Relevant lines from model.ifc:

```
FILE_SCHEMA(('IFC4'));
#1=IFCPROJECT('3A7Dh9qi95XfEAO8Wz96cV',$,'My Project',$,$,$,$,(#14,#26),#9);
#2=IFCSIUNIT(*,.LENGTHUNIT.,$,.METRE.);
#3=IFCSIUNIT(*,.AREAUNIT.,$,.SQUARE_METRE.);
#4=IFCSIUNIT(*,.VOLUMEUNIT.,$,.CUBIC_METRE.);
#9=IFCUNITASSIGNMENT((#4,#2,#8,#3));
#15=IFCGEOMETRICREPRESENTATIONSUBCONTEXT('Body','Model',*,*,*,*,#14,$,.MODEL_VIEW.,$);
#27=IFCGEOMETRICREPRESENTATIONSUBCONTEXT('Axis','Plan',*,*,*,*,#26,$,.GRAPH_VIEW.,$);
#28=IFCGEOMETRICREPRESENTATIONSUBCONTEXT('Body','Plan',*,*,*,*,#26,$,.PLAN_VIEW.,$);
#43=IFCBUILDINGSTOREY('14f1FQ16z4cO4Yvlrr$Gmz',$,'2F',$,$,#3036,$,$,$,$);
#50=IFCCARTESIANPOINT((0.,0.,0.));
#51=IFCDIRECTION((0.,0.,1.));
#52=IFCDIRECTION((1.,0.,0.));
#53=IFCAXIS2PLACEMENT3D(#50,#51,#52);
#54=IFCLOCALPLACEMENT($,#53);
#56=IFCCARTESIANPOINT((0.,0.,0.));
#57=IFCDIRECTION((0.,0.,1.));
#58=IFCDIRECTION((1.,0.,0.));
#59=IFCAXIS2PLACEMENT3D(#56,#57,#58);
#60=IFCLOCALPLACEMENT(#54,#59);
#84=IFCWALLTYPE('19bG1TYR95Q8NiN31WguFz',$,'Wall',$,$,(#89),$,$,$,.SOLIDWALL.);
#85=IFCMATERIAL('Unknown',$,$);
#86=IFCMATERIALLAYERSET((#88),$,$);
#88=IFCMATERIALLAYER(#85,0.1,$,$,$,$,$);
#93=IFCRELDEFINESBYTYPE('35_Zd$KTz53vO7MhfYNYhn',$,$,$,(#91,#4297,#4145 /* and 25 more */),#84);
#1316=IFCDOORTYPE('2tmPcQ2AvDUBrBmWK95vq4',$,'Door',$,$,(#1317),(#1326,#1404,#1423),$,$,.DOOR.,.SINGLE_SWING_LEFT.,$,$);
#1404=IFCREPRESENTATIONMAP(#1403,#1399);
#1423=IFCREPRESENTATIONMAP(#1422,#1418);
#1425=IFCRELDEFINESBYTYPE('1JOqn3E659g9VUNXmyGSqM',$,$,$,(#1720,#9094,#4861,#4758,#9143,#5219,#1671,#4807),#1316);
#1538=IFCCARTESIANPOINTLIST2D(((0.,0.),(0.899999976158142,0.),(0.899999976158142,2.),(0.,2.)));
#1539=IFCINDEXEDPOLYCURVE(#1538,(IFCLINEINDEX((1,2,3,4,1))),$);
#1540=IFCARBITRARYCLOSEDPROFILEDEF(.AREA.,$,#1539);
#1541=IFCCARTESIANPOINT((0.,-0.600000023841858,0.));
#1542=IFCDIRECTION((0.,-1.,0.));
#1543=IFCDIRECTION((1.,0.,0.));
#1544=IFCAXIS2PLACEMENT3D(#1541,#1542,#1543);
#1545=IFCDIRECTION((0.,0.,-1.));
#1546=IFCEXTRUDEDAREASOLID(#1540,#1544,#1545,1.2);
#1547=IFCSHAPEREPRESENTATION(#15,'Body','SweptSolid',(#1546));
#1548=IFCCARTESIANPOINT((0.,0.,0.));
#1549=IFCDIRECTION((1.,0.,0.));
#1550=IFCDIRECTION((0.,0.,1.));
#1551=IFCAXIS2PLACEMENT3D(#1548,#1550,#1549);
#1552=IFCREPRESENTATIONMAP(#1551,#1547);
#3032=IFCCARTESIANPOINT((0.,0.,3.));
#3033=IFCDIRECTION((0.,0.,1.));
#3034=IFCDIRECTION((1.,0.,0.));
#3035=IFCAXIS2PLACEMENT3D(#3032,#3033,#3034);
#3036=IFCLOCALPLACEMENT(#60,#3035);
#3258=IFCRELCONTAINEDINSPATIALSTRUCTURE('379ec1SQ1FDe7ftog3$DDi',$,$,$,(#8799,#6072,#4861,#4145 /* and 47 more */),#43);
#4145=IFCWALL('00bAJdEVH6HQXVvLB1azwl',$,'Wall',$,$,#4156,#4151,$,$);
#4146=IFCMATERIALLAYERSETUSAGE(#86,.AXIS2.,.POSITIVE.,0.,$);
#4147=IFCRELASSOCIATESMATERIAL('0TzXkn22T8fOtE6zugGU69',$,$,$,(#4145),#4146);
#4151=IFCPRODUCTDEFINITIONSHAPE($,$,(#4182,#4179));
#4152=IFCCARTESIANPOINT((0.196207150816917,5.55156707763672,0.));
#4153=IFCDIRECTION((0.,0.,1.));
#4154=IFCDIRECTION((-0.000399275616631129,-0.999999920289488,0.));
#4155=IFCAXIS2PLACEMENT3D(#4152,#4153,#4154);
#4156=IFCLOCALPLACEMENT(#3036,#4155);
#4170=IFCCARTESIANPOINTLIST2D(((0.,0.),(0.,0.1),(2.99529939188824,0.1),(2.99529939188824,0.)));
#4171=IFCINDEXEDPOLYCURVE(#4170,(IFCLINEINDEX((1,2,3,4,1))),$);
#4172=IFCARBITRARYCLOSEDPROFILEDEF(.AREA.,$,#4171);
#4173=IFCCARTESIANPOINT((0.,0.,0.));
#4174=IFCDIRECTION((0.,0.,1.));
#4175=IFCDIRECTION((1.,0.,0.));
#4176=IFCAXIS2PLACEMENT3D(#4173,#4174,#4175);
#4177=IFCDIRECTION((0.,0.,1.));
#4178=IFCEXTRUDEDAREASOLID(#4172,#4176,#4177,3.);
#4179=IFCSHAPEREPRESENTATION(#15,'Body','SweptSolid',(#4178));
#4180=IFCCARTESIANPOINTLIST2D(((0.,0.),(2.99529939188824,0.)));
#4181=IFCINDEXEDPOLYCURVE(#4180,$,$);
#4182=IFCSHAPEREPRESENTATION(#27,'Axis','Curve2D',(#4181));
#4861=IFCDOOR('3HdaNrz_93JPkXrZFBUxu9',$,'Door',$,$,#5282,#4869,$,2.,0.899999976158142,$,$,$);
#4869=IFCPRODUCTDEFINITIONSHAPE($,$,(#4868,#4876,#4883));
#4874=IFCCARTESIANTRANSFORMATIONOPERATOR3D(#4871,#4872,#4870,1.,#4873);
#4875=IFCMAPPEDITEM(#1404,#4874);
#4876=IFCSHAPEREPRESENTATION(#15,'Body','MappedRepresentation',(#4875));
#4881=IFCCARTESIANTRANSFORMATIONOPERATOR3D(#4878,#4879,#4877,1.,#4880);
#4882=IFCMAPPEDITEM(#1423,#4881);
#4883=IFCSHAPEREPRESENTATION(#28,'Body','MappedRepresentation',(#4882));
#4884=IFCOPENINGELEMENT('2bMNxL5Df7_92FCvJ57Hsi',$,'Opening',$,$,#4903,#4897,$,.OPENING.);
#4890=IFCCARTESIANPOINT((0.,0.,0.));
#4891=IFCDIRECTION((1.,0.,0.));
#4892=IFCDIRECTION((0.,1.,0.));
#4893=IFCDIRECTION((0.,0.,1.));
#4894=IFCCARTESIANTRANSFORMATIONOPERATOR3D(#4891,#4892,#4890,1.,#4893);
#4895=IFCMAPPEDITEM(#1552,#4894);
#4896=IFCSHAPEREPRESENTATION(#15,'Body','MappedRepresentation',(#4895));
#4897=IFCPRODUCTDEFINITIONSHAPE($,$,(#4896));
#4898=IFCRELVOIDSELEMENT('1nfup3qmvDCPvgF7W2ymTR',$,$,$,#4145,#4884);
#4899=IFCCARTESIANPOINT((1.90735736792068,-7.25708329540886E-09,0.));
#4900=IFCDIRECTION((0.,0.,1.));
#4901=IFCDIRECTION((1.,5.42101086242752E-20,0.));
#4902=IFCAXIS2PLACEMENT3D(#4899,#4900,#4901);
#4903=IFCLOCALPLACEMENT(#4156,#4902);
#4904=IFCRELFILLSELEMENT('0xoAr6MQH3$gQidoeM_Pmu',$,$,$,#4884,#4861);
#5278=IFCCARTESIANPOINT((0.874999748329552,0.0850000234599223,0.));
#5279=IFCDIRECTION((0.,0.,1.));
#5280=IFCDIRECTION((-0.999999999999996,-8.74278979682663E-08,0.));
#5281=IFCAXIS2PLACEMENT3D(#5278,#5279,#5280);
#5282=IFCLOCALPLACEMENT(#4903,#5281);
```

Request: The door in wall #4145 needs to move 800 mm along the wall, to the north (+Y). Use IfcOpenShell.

```python
import ifcopenshell
import ifcopenshell.api.geometry
import ifcopenshell.util.placement
import ifcopenshell.util.unit

model = ifcopenshell.open("model.ifc")
unit_scale = ifcopenshell.util.unit.calculate_unit_scale(model)

door = model.by_id(4861)
opening = door.FillsVoids[0].RelatingOpeningElement
wall = opening.VoidsElements[0].RelatingBuildingElement

wall_matrix = ifcopenshell.util.placement.get_local_placement(wall.ObjectPlacement)
shift = wall_matrix[:3, 0] * -0.8 / unit_scale
before = ifcopenshell.util.placement.get_local_placement(door.ObjectPlacement)[:3, 3].copy()

# The door is placed relative to its opening, so it follows when the opening moves.
matrix = ifcopenshell.util.placement.get_local_placement(opening.ObjectPlacement)
matrix[:3, 3] += shift
ifcopenshell.api.geometry.edit_object_placement(
    model, product=opening, matrix=matrix, is_si=False, should_transform_children=True
)

after = ifcopenshell.util.placement.get_local_placement(door.ObjectPlacement)[:3, 3]
print("door moved by", (after - before).round(3) + 0.0)

model.write("model_edited.ifc")
```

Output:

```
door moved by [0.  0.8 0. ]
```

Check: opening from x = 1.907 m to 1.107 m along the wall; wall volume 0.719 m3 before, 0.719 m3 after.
